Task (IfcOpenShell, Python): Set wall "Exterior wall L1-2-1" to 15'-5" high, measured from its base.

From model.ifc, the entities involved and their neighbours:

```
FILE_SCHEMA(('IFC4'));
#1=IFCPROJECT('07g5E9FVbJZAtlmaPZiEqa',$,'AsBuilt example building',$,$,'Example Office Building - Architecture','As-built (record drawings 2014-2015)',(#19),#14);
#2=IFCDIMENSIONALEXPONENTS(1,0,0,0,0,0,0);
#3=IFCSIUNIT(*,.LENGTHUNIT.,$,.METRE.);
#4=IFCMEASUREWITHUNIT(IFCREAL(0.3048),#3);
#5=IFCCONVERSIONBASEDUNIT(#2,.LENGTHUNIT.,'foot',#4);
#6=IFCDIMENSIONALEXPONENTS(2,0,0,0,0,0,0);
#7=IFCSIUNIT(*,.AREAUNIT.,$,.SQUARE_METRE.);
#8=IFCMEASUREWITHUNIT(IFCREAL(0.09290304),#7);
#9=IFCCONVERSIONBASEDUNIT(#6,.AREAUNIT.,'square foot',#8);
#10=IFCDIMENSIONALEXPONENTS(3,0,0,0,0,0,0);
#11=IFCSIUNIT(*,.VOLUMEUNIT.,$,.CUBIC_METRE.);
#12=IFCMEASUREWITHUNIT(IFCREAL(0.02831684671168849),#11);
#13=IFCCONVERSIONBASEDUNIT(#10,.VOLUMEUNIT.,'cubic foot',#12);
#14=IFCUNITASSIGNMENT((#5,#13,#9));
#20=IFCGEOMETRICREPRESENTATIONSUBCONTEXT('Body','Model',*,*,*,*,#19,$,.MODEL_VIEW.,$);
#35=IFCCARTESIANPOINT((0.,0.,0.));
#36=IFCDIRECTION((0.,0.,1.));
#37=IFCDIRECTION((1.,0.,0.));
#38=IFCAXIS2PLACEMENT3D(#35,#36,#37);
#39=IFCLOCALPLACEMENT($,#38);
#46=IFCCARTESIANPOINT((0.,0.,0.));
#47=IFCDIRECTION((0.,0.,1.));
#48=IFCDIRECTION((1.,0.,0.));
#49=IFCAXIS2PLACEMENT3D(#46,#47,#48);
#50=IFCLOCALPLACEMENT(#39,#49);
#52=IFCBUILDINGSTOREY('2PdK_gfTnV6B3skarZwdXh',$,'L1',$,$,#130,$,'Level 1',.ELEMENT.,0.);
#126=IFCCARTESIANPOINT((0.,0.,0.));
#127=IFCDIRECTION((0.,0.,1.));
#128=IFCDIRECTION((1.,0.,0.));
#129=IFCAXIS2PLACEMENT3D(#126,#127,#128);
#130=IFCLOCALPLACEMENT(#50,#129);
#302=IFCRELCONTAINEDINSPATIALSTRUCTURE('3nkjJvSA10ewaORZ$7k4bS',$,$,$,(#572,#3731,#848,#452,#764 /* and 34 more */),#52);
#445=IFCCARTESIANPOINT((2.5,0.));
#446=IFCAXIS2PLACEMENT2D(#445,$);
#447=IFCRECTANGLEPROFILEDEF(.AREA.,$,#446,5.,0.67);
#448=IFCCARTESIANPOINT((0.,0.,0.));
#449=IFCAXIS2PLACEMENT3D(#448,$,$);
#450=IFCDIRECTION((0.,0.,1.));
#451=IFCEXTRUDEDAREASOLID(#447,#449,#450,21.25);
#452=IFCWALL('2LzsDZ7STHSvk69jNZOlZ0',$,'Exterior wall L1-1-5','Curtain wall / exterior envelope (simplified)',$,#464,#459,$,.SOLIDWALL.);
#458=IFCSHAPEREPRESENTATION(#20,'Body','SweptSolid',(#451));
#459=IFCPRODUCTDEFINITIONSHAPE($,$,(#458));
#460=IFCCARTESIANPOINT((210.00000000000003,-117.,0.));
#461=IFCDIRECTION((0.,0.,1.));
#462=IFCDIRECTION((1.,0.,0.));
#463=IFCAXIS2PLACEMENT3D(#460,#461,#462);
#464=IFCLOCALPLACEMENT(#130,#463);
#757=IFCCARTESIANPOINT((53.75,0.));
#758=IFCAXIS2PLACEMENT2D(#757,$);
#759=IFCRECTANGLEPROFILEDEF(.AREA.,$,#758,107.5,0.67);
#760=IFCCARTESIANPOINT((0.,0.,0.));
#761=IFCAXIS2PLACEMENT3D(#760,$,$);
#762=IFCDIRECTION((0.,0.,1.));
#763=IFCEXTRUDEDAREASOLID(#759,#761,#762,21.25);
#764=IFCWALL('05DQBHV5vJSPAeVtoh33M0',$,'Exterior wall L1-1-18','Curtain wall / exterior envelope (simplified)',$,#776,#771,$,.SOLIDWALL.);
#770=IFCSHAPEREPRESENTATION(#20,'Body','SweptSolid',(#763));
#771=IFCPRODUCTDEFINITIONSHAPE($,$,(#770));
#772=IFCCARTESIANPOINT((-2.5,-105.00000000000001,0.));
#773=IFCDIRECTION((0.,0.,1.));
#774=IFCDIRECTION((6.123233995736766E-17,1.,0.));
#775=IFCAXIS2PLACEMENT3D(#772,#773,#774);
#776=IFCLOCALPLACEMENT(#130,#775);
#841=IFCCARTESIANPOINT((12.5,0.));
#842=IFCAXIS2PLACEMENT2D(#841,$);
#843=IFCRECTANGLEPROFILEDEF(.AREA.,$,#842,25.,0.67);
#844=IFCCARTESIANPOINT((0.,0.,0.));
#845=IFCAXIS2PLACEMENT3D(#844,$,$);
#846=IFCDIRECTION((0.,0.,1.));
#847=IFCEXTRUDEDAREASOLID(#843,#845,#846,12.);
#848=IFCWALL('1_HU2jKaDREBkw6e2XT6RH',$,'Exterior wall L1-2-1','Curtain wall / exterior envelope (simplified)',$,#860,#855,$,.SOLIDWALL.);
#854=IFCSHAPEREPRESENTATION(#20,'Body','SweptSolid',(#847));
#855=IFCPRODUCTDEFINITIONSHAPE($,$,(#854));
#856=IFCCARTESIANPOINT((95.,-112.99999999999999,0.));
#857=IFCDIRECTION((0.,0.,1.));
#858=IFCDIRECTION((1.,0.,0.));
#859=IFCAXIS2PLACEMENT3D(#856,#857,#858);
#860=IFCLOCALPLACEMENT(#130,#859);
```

```python
import ifcopenshell
import ifcopenshell.geom
import ifcopenshell.util.representation
import ifcopenshell.util.shape
import ifcopenshell.util.unit

model = ifcopenshell.open("model.ifc")
unit_scale = ifcopenshell.util.unit.calculate_unit_scale(model)
settings = ifcopenshell.geom.settings()


def volume(element):
    """Net volume in cubic metres, openings subtracted."""
    shape = ifcopenshell.geom.create_shape(settings, element)
    return ifcopenshell.util.shape.get_volume(shape.geometry)


wall = model.by_guid("1_HU2jKaDREBkw6e2XT6RH")
before = volume(wall)

body = ifcopenshell.util.representation.get_representation(wall, "Model", "Body")
solid = body.Items[0]
old_height = solid.Depth
solid.Depth = 185 * 0.0254 / unit_scale
after = volume(wall)

print(f"height {old_height:g} -> {solid.Depth:g}, volume {before:.3f} -> {after:.3f} m3")

model.write("model_v2.ifc")
```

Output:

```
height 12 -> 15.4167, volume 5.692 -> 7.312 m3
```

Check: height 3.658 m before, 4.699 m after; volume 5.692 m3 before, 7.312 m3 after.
